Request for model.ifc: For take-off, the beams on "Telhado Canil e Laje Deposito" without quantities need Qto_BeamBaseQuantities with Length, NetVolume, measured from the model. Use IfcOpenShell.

First a look at what the model holds.

```python
import ifcopenshell
import ifcopenshell.util.element
import ifcopenshell.util.unit

model = ifcopenshell.open("model.ifc")
print(model.schema)
for unit_type in ("LENGTHUNIT", "AREAUNIT", "VOLUMEUNIT"):
    print(unit_type, ifcopenshell.util.unit.calculate_unit_scale(model, unit_type))
storey = next(s for s in model.by_type("IfcBuildingStorey") if s.Name == "Telhado Canil e Laje Deposito")
beams = [e for e in ifcopenshell.util.element.get_decomposition(storey) if e.is_a("IfcBeam")]
for e in sorted(beams, key=lambda e: e.id()):
    print(e.id(), e.is_a(), e.Name, list(ifcopenshell.util.element.get_psets(e, qtos_only=True)), sep=" | ")
```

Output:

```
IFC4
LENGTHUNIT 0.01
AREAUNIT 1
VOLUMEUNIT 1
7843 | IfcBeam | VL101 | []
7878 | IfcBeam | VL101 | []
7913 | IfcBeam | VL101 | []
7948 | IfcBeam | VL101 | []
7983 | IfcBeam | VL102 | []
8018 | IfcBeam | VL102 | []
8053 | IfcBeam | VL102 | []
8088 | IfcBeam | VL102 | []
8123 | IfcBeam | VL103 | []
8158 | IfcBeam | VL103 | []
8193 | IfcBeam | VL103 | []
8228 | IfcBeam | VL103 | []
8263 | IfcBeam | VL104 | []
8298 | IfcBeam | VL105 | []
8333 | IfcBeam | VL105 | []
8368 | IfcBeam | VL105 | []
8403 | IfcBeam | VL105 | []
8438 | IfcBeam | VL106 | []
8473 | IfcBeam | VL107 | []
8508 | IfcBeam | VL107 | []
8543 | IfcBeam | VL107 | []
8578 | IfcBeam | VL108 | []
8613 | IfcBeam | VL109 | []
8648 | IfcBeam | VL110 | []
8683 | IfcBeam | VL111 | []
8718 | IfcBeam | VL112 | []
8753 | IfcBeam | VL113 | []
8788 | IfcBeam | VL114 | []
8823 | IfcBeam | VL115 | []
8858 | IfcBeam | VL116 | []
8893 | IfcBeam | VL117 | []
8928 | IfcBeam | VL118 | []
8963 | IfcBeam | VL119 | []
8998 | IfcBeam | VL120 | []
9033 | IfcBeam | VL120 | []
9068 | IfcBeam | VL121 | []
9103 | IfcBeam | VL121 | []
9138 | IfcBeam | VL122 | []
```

```python
import ifcopenshell
import ifcopenshell.api.pset
import ifcopenshell.geom
import ifcopenshell.util.element
import ifcopenshell.util.shape
import ifcopenshell.util.unit

model = ifcopenshell.open("model.ifc")
unit_scale = ifcopenshell.util.unit.calculate_unit_scale(model)
volume_scale = ifcopenshell.util.unit.calculate_unit_scale(model, "VOLUMEUNIT")
settings = ifcopenshell.geom.settings()

storey = next(s for s in model.by_type("IfcBuildingStorey") if s.Name == "Telhado Canil e Laje Deposito")
beams = [e for e in ifcopenshell.util.element.get_decomposition(storey) if e.is_a("IfcBeam")]

for e in sorted(beams, key=lambda e: e.id()):
    if ifcopenshell.util.element.get_psets(e, qtos_only=True, should_inherit=False):
        continue
    # Geometry comes back in metres, in the element's own axes.
    shape = ifcopenshell.geom.create_shape(settings, e)
    values = {
        "Length": ifcopenshell.util.shape.get_max_xyz(shape.geometry) / unit_scale,
        "NetVolume": ifcopenshell.util.shape.get_volume(shape.geometry) / volume_scale,
    }
    qto = ifcopenshell.api.pset.add_qto(model, product=e, name="Qto_BeamBaseQuantities")
    ifcopenshell.api.pset.edit_qto(model, qto=qto, properties=values)
    print(e.id(), {k: round(v, 3) for k, v in values.items()})

model.write("model_rev.ifc")
```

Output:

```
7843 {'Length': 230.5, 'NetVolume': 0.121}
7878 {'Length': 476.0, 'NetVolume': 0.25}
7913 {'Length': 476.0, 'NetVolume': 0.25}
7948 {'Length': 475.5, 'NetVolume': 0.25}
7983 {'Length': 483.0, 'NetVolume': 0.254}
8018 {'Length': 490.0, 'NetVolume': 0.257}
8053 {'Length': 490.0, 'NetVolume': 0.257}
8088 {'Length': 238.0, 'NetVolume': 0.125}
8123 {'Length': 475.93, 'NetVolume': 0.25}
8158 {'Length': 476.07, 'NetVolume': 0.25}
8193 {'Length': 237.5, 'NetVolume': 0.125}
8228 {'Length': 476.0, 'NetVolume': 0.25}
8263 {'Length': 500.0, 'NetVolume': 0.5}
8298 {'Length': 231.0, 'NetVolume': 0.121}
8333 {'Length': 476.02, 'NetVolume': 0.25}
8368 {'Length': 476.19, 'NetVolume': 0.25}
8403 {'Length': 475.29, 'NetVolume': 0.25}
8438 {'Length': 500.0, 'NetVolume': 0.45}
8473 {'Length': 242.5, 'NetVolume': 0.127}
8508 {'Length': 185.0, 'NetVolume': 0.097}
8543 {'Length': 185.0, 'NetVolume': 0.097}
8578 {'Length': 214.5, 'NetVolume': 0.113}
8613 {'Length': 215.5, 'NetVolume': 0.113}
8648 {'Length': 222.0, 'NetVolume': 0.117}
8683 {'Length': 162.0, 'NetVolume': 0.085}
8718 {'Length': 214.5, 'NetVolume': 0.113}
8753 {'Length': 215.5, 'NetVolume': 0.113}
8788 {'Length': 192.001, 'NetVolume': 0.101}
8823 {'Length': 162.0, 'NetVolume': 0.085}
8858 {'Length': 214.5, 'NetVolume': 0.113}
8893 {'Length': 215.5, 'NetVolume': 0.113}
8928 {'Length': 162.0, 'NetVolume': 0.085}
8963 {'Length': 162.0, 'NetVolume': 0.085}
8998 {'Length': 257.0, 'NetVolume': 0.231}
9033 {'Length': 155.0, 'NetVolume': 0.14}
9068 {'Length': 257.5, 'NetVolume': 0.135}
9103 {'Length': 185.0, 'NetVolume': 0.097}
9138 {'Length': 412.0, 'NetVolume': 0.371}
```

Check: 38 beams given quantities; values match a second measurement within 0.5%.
